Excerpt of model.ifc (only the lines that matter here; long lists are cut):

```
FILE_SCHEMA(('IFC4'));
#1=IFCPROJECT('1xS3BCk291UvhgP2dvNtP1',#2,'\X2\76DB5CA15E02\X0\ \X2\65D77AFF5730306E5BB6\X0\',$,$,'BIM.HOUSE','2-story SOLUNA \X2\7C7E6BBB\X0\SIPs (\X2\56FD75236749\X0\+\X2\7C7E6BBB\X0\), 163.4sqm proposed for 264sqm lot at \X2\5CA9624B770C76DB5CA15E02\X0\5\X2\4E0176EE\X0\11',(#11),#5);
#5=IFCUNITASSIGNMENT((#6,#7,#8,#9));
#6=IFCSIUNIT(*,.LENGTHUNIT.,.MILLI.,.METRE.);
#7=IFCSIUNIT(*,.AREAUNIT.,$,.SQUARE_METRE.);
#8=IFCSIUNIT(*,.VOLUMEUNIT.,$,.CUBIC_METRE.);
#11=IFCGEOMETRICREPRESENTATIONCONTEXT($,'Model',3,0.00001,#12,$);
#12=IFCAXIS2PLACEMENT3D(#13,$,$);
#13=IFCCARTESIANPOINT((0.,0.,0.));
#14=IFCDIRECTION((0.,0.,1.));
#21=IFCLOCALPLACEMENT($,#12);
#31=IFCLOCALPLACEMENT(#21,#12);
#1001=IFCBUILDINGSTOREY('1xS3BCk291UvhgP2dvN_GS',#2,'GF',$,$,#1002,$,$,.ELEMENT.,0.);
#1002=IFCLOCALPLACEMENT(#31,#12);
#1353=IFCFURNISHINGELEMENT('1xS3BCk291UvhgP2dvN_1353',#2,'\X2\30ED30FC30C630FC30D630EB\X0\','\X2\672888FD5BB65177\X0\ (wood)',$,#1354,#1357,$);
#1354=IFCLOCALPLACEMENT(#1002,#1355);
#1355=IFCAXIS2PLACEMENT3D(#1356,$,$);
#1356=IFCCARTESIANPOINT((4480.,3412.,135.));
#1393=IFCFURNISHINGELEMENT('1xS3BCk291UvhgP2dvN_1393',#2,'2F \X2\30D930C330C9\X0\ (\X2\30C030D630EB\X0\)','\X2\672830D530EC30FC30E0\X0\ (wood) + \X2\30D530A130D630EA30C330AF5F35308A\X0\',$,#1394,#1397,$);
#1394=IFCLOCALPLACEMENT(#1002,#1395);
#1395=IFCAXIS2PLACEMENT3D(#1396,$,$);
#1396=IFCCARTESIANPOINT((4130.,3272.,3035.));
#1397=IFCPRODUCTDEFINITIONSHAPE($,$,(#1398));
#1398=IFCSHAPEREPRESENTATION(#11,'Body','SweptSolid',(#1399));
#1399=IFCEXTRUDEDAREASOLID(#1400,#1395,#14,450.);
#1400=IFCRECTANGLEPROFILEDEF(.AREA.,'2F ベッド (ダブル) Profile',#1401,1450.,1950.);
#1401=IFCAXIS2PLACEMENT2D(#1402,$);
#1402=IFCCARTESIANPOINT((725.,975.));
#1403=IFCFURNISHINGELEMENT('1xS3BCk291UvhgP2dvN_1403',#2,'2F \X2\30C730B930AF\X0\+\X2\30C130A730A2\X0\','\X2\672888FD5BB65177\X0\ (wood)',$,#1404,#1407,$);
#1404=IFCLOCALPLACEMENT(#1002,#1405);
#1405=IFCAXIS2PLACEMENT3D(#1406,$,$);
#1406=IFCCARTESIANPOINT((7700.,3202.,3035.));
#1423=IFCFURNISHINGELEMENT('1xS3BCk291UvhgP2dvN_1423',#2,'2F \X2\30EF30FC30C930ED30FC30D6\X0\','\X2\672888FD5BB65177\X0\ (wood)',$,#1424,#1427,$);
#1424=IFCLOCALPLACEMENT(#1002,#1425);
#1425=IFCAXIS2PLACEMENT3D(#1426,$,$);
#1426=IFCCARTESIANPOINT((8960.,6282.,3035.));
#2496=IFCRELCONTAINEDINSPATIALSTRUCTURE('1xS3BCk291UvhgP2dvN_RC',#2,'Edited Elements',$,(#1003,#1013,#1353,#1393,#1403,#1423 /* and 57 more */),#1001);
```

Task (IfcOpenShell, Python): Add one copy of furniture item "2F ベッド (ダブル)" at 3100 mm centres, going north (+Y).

```python
import numpy as np
import ifcopenshell
import ifcopenshell.api.geometry
import ifcopenshell.api.root
import ifcopenshell.util.element
import ifcopenshell.util.placement

model = ifcopenshell.open("model.ifc")


def reuse_history(source, copy):
    """copy_class also copies each property set's owner history, people and application; keep the originals."""
    for rel in copy.IsDefinedBy:
        if rel.is_a("IfcRelDefinesByProperties") and (history := rel.RelatingPropertyDefinition.OwnerHistory):
            rel.RelatingPropertyDefinition.OwnerHistory = source.OwnerHistory
            ifcopenshell.util.element.remove_deep2(model, history)


source = model.by_id(1393)
base = ifcopenshell.util.placement.get_local_placement(source.ObjectPlacement)
step = np.array([0.0, 1.0, 0.0]) * 3100.0

for i in range(1, 2):
    copy = ifcopenshell.api.root.copy_class(model, product=source)
    copy.Representation = ifcopenshell.util.element.copy_deep(
        model, source.Representation, exclude=["IfcGeometricRepresentationContext", "IfcRepresentationMap"]
    )
    reuse_history(source, copy)
    matrix = base.copy()
    matrix[:3, 3] += i * step
    print("added at", matrix[:3, 3].round(3) + 0.0)
    ifcopenshell.api.geometry.edit_object_placement(model, product=copy, matrix=matrix, is_si=False)

model.write("model_updated.ifc")
```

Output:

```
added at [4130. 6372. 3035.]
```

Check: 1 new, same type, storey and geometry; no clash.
